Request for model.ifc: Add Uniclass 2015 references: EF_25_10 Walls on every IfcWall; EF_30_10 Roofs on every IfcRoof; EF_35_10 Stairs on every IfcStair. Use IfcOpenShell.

First a look at what the model holds.

```python
import ifcopenshell

model = ifcopenshell.open("model.ifc")
print(model.schema)
print("classifications:", [c.Name for c in model.by_type("IfcClassification")])
for ifc_class in ("IfcDoor", "IfcRoof", "IfcStair", "IfcWall", "IfcWindow"):
    print(ifc_class, len(model.by_type(ifc_class)))
```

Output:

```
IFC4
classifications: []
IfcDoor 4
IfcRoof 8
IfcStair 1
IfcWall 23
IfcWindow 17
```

```python
import ifcopenshell
import ifcopenshell.api.classification

model = ifcopenshell.open("model.ifc")

system = ifcopenshell.api.classification.add_classification(model, classification="Uniclass 2015")

codes = {
    "IfcWall": ("EF_25_10", "Walls"),
    "IfcRoof": ("EF_30_10", "Roofs"),
    "IfcStair": ("EF_35_10", "Stairs"),
}
for ifc_class, (code, name) in codes.items():
    products = model.by_type(ifc_class)
    ifcopenshell.api.classification.add_reference(
        model, products=products, classification=system, identification=code, name=name
    )
    print(code, len(products))

model.write("model_rev.ifc")
```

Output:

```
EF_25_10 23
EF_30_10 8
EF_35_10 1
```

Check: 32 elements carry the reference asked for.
